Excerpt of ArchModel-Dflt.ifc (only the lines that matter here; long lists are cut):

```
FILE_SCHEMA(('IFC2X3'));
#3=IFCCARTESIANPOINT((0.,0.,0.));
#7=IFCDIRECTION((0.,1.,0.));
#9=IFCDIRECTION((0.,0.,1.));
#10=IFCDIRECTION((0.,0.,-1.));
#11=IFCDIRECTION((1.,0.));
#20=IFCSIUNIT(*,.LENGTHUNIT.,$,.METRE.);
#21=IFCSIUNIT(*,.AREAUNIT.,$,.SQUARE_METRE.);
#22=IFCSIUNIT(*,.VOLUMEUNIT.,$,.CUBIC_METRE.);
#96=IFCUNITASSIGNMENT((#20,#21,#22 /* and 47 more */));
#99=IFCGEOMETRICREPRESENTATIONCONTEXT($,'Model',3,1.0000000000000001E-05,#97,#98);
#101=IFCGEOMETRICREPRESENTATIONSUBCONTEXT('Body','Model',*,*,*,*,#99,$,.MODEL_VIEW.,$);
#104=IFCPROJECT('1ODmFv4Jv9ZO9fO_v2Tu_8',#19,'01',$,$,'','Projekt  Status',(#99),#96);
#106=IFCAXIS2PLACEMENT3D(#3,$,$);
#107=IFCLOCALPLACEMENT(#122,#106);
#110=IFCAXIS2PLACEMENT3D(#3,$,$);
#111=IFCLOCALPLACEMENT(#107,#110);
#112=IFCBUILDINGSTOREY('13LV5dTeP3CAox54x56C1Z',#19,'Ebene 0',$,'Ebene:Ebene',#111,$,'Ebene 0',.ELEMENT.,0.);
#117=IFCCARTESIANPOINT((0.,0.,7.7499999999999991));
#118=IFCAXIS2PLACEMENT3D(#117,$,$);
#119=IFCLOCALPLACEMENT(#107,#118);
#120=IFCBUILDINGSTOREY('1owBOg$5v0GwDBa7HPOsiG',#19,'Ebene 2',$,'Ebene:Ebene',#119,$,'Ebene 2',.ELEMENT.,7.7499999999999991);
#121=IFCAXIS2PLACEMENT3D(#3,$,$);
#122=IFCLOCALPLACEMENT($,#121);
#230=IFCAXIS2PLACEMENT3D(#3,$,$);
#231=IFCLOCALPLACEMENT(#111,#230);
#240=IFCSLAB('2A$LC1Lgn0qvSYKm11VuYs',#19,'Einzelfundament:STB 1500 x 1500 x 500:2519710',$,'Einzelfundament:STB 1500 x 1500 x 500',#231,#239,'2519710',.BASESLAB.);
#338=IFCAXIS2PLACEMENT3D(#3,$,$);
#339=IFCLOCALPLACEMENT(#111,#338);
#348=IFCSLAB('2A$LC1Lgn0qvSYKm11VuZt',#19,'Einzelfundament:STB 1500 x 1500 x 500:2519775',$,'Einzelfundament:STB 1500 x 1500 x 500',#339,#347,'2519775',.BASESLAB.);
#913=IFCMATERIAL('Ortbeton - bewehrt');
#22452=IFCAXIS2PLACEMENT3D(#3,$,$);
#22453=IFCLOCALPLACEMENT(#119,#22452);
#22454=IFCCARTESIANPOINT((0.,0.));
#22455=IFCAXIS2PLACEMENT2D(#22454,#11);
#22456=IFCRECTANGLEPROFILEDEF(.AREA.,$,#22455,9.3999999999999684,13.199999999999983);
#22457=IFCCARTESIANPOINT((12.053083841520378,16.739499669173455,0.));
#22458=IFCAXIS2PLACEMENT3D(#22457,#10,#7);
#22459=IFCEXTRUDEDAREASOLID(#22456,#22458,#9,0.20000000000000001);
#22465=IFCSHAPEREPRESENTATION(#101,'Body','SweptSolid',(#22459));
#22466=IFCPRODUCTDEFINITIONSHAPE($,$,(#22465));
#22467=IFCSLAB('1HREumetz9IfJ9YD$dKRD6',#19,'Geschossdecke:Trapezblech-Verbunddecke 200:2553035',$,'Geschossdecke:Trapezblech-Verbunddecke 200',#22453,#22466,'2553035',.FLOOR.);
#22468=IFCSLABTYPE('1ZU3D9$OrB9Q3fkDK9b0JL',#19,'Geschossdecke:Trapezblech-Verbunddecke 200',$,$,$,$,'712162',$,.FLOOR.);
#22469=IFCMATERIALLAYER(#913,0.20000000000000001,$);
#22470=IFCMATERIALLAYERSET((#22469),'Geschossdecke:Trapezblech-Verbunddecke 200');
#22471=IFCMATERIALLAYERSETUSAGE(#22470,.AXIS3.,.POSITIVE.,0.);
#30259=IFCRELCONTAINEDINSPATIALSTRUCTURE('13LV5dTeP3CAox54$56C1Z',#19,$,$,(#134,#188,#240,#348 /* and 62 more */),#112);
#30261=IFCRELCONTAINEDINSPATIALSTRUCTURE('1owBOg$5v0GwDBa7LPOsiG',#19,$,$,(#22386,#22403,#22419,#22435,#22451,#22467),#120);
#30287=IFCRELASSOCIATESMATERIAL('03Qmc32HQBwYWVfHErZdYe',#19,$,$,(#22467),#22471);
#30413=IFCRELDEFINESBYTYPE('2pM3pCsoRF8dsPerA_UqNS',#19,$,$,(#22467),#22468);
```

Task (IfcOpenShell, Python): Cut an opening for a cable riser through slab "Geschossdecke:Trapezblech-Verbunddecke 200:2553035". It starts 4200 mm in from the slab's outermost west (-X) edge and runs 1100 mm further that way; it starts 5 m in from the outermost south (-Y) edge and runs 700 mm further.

```python
import numpy as np
import ifcopenshell
import ifcopenshell.api.feature
import ifcopenshell.api.geometry
import ifcopenshell.api.root
import ifcopenshell.geom
import ifcopenshell.util.placement
import ifcopenshell.util.representation
import ifcopenshell.util.shape
import ifcopenshell.util.unit

model = ifcopenshell.open("ArchModel-Dflt.ifc")
unit_scale = ifcopenshell.util.unit.calculate_unit_scale(model)
settings = ifcopenshell.geom.settings()


def volume(element):
    """Net volume in cubic metres, openings subtracted."""
    shape = ifcopenshell.geom.create_shape(settings, element)
    return ifcopenshell.util.shape.get_volume(shape.geometry)


slab = model.by_guid("1HREumetz9IfJ9YD$dKRD6")
before = volume(slab)

# Extent in the slab's own axes, in metres. The edges named are its -X and -Y sides.
slab_shape = ifcopenshell.geom.create_shape(settings, slab)
vertices = ifcopenshell.util.shape.get_vertices(slab_shape.geometry)
x_min, y_min, bottom = vertices.min(axis=0)
top = vertices[:, 2].max()

opening = ifcopenshell.api.root.create_entity(model, ifc_class="IfcOpeningElement", name="Cable riser opening")
context = ifcopenshell.util.representation.get_context(model, "Model", "Body", "MODEL_VIEW")
width, depth = 1.1, 0.7
outline = [(0.0, 0.0), (width, 0.0), (width, depth), (0.0, depth), (0.0, 0.0)]
# Overshoot both faces by 50 mm so the cut is clean.
shape = ifcopenshell.api.geometry.add_slab_representation(
    model, context=context, depth=top - bottom + 0.1, polyline=outline
)
ifcopenshell.api.geometry.assign_representation(model, product=opening, representation=shape)

matrix = ifcopenshell.util.placement.get_local_placement(slab.ObjectPlacement)
matrix[:, 3] = matrix @ np.append(np.array([x_min + 4.2, y_min + 5, bottom - 0.05]) / unit_scale, 1.0)
ifcopenshell.api.geometry.edit_object_placement(model, product=opening, matrix=matrix, is_si=False)
ifcopenshell.api.feature.add_feature(model, feature=opening, element=slab)

after = volume(slab)

print(f"slab volume {before:.3f} -> {after:.3f} m3")

model.write("ArchModel-Dflt_updated.ifc")
```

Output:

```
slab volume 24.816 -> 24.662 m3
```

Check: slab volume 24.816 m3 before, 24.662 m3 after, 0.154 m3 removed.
